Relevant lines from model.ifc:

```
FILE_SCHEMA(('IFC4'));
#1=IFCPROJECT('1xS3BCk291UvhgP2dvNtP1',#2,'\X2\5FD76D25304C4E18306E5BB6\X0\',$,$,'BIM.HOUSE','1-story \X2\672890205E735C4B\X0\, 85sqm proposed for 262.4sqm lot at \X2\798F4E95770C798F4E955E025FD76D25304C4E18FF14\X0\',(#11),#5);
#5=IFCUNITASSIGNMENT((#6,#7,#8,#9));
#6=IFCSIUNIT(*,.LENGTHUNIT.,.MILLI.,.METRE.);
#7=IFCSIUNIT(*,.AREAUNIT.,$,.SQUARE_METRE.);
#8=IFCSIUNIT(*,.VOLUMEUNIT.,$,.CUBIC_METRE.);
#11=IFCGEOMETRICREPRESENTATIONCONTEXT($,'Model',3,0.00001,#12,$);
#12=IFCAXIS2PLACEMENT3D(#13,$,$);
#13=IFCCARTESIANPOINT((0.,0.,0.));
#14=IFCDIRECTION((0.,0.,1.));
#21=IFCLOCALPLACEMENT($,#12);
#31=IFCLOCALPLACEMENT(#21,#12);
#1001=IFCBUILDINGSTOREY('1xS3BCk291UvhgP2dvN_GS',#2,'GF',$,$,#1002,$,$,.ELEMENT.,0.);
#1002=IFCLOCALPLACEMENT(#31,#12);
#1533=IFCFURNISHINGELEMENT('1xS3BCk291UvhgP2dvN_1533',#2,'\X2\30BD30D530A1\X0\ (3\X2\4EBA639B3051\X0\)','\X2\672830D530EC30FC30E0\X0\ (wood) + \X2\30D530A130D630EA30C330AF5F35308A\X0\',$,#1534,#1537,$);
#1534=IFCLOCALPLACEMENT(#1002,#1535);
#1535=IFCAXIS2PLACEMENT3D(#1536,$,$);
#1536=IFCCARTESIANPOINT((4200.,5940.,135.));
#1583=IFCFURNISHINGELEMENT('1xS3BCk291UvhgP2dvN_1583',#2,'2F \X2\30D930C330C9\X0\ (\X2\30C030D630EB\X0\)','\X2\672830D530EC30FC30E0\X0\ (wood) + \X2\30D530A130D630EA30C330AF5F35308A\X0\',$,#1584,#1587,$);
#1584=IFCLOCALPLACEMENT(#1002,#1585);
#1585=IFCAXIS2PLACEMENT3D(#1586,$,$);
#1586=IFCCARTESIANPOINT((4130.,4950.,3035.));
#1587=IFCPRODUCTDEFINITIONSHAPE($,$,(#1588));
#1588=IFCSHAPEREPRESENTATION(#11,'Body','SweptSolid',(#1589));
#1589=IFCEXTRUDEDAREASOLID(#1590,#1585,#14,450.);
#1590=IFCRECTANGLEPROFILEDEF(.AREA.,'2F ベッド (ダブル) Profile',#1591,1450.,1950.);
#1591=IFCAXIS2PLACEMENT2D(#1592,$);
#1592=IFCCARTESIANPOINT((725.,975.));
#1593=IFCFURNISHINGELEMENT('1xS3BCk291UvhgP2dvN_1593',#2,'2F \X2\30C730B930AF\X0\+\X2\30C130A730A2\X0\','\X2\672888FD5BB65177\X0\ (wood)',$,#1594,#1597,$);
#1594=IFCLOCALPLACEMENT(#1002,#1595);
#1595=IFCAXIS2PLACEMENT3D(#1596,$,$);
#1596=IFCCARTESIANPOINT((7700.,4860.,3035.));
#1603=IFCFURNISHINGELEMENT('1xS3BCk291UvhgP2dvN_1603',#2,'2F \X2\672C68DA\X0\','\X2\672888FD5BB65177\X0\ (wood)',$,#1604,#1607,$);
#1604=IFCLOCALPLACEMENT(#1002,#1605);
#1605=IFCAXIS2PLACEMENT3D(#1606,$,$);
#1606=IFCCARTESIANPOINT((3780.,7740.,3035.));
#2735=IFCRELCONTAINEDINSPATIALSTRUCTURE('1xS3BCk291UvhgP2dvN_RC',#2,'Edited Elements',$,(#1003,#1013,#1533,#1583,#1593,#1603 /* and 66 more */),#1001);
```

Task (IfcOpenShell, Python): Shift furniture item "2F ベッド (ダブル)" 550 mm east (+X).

```python
import ifcopenshell
import ifcopenshell.api.geometry
import ifcopenshell.util.placement

model = ifcopenshell.open("model.ifc")

item = model.by_guid("1xS3BCk291UvhgP2dvN_1583")
matrix = ifcopenshell.util.placement.get_local_placement(item.ObjectPlacement)
matrix[0, 3] += 550.0
ifcopenshell.api.geometry.edit_object_placement(model, product=item, matrix=matrix, is_si=False)

print(ifcopenshell.util.placement.get_local_placement(item.ObjectPlacement).round(3) + 0.0)

model.write("model_edited.ifc")
```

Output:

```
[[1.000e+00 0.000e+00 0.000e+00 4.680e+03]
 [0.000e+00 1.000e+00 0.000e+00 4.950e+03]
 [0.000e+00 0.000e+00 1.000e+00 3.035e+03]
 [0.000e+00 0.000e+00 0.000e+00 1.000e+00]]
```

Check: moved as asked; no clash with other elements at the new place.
